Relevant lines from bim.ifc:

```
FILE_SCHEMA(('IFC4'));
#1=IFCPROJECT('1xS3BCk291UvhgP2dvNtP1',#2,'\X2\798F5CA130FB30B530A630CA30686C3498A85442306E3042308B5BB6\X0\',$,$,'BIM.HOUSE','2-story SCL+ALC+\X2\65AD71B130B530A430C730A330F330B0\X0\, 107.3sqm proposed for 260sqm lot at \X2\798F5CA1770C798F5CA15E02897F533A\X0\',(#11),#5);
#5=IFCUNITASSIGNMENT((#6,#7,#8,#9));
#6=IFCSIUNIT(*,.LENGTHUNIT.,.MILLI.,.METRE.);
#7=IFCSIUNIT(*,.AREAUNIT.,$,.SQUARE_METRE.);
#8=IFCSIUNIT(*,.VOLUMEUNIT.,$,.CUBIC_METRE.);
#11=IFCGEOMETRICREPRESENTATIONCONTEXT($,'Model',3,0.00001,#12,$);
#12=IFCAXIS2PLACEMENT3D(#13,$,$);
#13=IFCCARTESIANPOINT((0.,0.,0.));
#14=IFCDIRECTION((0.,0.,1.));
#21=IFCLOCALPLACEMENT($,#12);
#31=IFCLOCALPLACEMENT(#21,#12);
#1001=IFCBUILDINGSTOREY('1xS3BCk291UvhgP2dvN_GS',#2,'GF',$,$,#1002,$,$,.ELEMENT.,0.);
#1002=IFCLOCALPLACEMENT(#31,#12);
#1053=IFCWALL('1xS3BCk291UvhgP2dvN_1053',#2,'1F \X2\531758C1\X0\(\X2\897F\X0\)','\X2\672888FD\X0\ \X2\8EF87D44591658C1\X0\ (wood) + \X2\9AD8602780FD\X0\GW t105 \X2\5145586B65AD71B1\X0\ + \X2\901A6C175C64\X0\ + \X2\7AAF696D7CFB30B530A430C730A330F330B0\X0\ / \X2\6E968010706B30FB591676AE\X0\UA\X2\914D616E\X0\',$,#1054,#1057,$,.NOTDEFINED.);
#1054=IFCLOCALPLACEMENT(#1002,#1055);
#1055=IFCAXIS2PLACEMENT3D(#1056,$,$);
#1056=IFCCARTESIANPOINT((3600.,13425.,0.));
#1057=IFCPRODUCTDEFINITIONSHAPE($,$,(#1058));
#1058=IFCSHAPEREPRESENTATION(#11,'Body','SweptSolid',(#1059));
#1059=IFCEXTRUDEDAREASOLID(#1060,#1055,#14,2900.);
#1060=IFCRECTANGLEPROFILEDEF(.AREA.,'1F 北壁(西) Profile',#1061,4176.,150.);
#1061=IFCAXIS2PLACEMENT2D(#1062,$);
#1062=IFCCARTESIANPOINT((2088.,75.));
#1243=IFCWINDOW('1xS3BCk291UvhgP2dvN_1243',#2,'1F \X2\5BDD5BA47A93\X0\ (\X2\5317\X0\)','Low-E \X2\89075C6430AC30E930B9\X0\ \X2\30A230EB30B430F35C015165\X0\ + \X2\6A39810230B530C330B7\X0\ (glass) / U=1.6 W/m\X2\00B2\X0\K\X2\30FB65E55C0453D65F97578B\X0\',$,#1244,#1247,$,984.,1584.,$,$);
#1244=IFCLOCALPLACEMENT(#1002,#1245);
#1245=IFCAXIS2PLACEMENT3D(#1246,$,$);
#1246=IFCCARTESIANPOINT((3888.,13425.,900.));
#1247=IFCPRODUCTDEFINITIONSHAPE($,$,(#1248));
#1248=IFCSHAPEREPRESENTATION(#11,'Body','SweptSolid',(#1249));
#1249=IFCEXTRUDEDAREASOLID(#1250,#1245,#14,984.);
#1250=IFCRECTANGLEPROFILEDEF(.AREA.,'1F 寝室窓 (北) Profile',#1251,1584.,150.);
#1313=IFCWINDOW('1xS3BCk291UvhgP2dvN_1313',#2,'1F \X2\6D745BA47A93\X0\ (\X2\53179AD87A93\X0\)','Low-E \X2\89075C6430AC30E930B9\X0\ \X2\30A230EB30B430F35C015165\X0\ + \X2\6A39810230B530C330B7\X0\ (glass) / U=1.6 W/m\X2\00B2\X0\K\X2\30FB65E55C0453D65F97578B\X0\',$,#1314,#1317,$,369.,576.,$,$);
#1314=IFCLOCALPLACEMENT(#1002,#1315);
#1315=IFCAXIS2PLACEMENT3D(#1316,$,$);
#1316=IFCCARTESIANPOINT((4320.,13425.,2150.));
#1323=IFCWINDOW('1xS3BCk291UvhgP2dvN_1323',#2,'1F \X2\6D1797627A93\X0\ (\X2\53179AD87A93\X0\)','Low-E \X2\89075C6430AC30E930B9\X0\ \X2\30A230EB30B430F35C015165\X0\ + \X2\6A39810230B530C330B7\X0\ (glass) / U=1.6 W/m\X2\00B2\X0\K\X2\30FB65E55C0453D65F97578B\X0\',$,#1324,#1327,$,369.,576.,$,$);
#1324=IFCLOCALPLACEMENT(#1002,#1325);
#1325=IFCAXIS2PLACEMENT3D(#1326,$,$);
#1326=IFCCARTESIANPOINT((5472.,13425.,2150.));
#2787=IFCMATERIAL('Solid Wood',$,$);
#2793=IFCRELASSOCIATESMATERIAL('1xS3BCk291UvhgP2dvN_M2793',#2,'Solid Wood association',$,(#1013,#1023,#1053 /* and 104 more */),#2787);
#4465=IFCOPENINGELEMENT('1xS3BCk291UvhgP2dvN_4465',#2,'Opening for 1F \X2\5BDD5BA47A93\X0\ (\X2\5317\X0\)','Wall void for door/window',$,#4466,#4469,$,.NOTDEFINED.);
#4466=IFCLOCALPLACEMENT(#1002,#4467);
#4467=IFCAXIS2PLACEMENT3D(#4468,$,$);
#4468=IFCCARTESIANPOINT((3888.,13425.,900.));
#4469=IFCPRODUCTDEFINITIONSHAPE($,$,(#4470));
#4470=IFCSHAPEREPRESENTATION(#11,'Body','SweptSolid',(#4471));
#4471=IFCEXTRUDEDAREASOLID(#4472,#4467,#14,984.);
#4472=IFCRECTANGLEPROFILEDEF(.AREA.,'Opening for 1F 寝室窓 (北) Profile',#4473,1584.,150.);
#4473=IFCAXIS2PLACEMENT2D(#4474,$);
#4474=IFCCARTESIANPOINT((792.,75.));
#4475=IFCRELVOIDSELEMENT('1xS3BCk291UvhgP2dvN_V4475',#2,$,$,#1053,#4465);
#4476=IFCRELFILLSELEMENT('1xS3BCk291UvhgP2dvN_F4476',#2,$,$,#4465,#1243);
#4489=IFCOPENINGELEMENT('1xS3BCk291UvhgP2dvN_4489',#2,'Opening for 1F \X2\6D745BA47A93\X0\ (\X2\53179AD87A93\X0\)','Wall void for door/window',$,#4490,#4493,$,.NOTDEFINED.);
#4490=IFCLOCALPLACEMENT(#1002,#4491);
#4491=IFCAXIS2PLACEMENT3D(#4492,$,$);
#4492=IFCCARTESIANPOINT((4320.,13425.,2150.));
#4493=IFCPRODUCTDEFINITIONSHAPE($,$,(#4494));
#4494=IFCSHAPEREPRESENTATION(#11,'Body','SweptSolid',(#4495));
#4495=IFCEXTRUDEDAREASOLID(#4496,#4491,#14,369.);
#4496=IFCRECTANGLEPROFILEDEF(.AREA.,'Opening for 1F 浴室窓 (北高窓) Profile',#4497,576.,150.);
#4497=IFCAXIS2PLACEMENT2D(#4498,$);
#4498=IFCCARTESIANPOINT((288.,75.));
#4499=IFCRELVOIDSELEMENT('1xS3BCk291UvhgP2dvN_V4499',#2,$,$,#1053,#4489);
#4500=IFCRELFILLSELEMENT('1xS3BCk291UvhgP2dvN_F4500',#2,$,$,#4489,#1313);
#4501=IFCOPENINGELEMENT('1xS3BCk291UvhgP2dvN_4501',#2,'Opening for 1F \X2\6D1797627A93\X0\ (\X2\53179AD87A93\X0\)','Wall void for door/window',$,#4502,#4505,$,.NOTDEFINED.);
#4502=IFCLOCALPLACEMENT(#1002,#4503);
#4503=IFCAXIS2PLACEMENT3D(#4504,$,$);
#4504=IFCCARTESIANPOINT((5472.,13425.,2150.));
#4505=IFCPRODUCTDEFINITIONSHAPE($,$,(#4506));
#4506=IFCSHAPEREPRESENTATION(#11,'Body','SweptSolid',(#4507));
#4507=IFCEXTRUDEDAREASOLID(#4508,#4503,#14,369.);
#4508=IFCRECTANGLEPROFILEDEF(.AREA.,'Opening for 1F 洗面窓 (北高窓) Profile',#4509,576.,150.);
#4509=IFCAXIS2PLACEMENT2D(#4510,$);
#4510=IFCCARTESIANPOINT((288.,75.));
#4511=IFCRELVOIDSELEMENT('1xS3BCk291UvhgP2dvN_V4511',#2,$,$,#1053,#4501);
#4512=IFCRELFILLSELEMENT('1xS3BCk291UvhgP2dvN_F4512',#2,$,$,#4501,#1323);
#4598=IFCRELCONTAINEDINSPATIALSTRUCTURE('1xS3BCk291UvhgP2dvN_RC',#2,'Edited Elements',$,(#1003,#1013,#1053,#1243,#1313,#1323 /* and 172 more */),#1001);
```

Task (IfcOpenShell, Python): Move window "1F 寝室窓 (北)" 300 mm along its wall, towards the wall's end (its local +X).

```python
import ifcopenshell
import ifcopenshell.api.geometry
import ifcopenshell.util.placement

model = ifcopenshell.open("bim.ifc")

window = model.by_id(1243)
opening = window.FillsVoids[0].RelatingOpeningElement
wall = opening.VoidsElements[0].RelatingBuildingElement

wall_matrix = ifcopenshell.util.placement.get_local_placement(wall.ObjectPlacement)
shift = wall_matrix[:3, 0] * 300.0
before = ifcopenshell.util.placement.get_local_placement(window.ObjectPlacement)[:3, 3].copy()

# The window is not placed relative to its opening, so move both.
for product in (opening, window):
    matrix = ifcopenshell.util.placement.get_local_placement(product.ObjectPlacement)
    matrix[:3, 3] += shift
    ifcopenshell.api.geometry.edit_object_placement(model, product=product, matrix=matrix, is_si=False)

after = ifcopenshell.util.placement.get_local_placement(window.ObjectPlacement)[:3, 3]
print("window moved by", (after - before).round(3) + 0.0)

model.write("bim_v2.ifc")
```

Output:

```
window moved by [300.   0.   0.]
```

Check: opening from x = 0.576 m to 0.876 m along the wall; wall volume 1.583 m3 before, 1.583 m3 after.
